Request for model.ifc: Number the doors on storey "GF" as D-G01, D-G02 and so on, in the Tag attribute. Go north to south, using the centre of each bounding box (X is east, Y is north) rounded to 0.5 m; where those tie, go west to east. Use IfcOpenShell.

First a look at what the model holds.

```python
import ifcopenshell
import ifcopenshell.util.element
import ifcopenshell.util.placement

model = ifcopenshell.open("model.ifc")
print(model.schema)
storey = next(s for s in model.by_type("IfcBuildingStorey") if s.Name == "GF")
doors = [e for e in ifcopenshell.util.element.get_decomposition(storey) if e.is_a("IfcDoor")]
for e in sorted(doors, key=lambda e: e.id()):
    origin = ifcopenshell.util.placement.get_local_placement(e.ObjectPlacement)[:3, 3]
    print(e.id(), e.Tag, e.Name, origin.round(2) + 0.0, sep=" | ")
```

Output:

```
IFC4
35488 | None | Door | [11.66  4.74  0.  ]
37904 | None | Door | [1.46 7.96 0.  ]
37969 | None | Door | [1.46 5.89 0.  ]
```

```python
import ifcopenshell
import ifcopenshell.geom
import ifcopenshell.util.element
import ifcopenshell.util.shape

model = ifcopenshell.open("model.ifc")
settings = ifcopenshell.geom.settings()
settings.set("use-world-coords", True)


def centre(element):
    shape = ifcopenshell.geom.create_shape(settings, element)
    return ifcopenshell.util.shape.get_bbox_centroid(shape.geometry)


storey = next(s for s in model.by_type("IfcBuildingStorey") if s.Name == "GF")
doors = [e for e in ifcopenshell.util.element.get_decomposition(storey) if e.is_a("IfcDoor")]

# Insertion points can sit at a corner or the storey origin, so sort by the geometry (in metres).
centres = {e: centre(e) for e in doors}
doors.sort(key=lambda e: (-round(centres[e][1] / 0.5), centres[e][0]))

for i, e in enumerate(doors, start=1):
    number = f"D-G{i:02d}"
    e.Tag = number
    print(e.id(), number)

model.write("model-out.ifc")
```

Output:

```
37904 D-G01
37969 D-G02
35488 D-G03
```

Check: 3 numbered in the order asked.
